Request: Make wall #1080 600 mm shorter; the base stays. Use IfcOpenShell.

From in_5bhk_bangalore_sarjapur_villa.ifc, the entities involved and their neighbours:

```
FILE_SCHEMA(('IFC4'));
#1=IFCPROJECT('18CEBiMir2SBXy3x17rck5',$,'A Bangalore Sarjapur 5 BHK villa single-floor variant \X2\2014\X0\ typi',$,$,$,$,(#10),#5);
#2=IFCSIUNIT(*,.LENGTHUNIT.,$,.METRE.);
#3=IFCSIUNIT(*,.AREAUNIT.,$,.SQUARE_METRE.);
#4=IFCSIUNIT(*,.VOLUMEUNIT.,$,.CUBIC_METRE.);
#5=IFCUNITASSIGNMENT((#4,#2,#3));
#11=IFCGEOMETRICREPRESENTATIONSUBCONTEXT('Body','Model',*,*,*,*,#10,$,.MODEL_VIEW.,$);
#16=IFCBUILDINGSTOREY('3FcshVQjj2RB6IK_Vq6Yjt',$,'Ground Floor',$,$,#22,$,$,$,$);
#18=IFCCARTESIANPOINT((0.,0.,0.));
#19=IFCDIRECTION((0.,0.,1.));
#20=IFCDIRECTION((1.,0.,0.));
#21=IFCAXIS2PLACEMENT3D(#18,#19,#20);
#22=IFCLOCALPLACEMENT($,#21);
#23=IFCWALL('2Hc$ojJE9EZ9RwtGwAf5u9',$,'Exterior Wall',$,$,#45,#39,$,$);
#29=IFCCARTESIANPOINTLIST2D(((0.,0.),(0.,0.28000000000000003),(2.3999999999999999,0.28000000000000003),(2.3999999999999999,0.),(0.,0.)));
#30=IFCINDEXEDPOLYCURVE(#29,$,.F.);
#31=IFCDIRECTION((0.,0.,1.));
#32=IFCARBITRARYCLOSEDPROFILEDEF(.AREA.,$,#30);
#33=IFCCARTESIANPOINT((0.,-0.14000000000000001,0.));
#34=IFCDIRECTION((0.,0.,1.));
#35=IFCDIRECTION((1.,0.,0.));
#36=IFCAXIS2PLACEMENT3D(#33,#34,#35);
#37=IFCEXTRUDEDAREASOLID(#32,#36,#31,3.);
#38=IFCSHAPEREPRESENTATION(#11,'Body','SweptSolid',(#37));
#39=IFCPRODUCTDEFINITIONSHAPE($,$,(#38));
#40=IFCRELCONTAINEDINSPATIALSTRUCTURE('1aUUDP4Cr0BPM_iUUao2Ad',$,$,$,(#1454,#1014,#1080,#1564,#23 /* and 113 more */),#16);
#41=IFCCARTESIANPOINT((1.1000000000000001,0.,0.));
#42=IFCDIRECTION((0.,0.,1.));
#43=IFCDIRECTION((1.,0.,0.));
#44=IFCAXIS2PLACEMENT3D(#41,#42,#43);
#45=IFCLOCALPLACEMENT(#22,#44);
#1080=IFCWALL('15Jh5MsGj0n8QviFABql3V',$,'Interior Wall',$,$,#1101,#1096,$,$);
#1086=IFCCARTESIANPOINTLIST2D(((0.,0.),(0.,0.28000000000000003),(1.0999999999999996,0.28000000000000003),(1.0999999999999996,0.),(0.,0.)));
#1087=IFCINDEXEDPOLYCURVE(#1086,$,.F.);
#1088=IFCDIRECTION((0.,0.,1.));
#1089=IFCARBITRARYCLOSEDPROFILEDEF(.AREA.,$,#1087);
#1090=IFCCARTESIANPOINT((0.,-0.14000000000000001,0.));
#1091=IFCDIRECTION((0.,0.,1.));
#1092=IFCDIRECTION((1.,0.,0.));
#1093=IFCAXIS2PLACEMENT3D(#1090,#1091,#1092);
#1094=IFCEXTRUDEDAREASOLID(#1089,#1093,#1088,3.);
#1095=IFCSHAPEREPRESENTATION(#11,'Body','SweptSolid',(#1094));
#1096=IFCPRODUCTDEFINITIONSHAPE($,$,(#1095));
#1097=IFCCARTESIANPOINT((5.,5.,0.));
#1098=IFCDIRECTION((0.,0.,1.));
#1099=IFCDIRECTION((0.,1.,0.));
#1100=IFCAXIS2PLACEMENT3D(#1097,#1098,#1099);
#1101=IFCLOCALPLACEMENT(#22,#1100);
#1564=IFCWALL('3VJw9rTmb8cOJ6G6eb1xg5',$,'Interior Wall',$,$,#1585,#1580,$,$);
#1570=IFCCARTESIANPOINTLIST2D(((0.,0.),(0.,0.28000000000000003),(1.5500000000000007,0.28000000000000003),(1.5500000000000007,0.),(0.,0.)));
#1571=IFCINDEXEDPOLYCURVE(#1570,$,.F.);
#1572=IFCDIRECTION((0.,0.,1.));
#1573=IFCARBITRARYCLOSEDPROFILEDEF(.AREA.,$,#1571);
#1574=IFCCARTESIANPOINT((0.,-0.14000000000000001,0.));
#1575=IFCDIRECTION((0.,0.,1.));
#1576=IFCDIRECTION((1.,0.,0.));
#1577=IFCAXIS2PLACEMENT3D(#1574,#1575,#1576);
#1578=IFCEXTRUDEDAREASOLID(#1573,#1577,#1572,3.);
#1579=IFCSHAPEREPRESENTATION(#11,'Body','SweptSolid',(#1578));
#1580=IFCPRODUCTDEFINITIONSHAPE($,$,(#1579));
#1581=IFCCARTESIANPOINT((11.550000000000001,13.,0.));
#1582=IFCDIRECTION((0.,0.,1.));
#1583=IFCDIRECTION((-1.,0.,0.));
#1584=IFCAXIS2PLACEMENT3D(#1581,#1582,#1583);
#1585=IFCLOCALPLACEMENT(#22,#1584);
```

```python
import ifcopenshell
import ifcopenshell.geom
import ifcopenshell.util.representation
import ifcopenshell.util.shape

model = ifcopenshell.open("in_5bhk_bangalore_sarjapur_villa.ifc")
settings = ifcopenshell.geom.settings()


def volume(element):
    """Net volume in cubic metres, openings subtracted."""
    shape = ifcopenshell.geom.create_shape(settings, element)
    return ifcopenshell.util.shape.get_volume(shape.geometry)


wall = model.by_guid("15Jh5MsGj0n8QviFABql3V")
before = volume(wall)

body = ifcopenshell.util.representation.get_representation(wall, "Model", "Body")
solid = body.Items[0]
old_height = solid.Depth
solid.Depth -= 0.6
after = volume(wall)

print(f"height {old_height:g} -> {solid.Depth:g}, volume {before:.3f} -> {after:.3f} m3")

model.write("in_5bhk_bangalore_sarjapur_villa_edited.ifc")
```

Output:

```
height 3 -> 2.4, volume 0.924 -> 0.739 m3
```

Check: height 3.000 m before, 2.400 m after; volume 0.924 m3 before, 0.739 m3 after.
